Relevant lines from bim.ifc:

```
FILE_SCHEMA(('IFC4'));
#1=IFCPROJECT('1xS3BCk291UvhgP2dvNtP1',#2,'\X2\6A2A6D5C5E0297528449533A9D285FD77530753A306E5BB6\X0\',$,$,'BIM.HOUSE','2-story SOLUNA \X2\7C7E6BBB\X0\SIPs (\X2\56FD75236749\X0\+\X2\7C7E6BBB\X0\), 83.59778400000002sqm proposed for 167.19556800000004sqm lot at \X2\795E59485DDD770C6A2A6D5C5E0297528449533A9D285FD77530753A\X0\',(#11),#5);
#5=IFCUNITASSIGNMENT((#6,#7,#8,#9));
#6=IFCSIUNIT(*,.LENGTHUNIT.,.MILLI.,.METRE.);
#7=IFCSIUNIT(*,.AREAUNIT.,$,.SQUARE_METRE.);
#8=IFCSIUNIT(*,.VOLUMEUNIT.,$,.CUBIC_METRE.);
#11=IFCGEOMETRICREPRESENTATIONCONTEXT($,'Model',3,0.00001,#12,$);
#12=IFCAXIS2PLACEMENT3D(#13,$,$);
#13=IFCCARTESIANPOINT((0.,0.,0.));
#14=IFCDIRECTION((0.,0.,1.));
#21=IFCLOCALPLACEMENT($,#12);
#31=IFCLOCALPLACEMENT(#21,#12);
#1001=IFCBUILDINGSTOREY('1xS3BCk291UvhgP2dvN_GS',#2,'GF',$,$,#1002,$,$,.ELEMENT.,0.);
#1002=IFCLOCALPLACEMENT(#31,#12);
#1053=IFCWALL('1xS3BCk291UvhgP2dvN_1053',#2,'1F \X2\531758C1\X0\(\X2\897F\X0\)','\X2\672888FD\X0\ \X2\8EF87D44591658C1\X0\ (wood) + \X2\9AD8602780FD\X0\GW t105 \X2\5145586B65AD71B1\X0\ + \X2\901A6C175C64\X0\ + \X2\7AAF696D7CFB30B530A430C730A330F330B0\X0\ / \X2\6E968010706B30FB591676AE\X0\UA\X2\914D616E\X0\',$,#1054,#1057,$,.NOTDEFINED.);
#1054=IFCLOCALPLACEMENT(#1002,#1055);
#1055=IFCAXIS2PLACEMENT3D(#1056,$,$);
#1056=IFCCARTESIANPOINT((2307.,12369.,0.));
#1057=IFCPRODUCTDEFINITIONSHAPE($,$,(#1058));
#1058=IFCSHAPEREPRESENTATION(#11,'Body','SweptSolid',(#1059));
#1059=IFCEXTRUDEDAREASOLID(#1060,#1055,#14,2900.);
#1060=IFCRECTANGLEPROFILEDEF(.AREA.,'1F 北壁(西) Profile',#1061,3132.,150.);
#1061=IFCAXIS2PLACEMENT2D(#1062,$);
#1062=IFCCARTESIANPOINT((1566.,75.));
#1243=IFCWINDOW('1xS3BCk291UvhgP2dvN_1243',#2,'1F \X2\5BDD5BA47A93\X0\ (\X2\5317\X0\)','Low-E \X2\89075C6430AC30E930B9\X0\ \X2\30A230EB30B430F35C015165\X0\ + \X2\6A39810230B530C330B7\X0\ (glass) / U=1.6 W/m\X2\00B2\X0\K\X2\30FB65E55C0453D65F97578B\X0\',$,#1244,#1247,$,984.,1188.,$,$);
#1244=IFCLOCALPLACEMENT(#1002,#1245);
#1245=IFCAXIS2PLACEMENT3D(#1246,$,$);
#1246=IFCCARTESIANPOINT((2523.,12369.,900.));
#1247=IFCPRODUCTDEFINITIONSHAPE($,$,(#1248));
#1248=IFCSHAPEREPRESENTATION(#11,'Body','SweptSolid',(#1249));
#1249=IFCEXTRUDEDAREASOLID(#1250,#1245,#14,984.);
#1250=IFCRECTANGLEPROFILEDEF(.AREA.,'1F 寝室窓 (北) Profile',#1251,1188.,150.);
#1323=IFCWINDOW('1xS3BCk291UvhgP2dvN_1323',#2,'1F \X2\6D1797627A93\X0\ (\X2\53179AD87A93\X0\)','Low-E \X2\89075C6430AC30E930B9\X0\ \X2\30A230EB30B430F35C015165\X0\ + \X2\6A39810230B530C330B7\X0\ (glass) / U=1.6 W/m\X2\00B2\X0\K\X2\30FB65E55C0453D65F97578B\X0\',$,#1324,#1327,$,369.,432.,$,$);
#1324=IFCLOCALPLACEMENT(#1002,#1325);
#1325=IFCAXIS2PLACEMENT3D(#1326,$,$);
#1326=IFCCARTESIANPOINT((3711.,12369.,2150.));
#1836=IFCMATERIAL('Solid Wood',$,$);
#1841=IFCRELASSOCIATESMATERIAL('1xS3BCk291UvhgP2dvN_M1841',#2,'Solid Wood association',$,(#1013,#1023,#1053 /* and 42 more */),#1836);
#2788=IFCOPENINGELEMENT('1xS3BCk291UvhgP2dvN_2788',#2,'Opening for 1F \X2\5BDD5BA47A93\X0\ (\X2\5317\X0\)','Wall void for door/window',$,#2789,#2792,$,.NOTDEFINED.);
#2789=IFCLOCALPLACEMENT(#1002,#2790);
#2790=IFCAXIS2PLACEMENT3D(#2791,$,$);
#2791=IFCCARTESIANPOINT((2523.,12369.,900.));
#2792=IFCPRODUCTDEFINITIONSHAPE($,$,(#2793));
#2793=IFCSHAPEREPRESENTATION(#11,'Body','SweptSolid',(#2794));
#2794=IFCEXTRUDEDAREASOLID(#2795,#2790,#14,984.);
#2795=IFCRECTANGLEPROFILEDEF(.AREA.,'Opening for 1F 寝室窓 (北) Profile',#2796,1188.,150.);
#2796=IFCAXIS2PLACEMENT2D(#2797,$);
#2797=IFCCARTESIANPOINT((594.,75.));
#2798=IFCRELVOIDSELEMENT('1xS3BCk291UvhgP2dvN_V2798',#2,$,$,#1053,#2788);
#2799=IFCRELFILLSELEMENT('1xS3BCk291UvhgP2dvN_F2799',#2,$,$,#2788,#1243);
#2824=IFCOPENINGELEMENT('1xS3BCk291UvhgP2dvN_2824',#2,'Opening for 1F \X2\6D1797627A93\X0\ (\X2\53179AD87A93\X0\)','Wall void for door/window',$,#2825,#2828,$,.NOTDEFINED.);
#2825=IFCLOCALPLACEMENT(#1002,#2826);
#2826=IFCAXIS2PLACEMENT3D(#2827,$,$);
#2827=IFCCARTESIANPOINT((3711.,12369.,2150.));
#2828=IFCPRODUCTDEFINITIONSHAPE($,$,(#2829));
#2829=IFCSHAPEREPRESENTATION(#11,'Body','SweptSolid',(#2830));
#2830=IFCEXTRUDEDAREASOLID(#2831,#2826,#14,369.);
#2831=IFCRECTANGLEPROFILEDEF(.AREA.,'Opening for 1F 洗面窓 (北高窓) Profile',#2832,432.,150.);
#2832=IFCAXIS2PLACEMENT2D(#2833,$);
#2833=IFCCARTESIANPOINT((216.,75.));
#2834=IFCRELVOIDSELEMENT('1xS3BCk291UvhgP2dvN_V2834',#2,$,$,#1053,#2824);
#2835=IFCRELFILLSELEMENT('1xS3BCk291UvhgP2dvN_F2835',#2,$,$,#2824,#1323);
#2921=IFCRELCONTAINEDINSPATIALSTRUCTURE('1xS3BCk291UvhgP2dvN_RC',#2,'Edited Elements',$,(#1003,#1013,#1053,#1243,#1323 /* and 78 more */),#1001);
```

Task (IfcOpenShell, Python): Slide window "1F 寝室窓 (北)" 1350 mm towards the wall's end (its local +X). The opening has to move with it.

```python
import ifcopenshell
import ifcopenshell.api.geometry
import ifcopenshell.util.placement
import ifcopenshell.util.unit

model = ifcopenshell.open("bim.ifc")
unit_scale = ifcopenshell.util.unit.calculate_unit_scale(model)

window = model.by_guid("1xS3BCk291UvhgP2dvN_1243")
opening = window.FillsVoids[0].RelatingOpeningElement
wall = opening.VoidsElements[0].RelatingBuildingElement

wall_matrix = ifcopenshell.util.placement.get_local_placement(wall.ObjectPlacement)
shift = wall_matrix[:3, 0] * 1.35 / unit_scale
before = ifcopenshell.util.placement.get_local_placement(window.ObjectPlacement)[:3, 3].copy()

# The window is not placed relative to its opening, so move both.
for product in (opening, window):
    matrix = ifcopenshell.util.placement.get_local_placement(product.ObjectPlacement)
    matrix[:3, 3] += shift
    ifcopenshell.api.geometry.edit_object_placement(model, product=product, matrix=matrix, is_si=False)

after = ifcopenshell.util.placement.get_local_placement(window.ObjectPlacement)[:3, 3]
print("window moved by", (after - before).round(3) + 0.0)

model.write("bim-out.ifc")
```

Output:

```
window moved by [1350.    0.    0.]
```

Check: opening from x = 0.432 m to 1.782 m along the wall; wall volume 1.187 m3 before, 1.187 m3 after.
